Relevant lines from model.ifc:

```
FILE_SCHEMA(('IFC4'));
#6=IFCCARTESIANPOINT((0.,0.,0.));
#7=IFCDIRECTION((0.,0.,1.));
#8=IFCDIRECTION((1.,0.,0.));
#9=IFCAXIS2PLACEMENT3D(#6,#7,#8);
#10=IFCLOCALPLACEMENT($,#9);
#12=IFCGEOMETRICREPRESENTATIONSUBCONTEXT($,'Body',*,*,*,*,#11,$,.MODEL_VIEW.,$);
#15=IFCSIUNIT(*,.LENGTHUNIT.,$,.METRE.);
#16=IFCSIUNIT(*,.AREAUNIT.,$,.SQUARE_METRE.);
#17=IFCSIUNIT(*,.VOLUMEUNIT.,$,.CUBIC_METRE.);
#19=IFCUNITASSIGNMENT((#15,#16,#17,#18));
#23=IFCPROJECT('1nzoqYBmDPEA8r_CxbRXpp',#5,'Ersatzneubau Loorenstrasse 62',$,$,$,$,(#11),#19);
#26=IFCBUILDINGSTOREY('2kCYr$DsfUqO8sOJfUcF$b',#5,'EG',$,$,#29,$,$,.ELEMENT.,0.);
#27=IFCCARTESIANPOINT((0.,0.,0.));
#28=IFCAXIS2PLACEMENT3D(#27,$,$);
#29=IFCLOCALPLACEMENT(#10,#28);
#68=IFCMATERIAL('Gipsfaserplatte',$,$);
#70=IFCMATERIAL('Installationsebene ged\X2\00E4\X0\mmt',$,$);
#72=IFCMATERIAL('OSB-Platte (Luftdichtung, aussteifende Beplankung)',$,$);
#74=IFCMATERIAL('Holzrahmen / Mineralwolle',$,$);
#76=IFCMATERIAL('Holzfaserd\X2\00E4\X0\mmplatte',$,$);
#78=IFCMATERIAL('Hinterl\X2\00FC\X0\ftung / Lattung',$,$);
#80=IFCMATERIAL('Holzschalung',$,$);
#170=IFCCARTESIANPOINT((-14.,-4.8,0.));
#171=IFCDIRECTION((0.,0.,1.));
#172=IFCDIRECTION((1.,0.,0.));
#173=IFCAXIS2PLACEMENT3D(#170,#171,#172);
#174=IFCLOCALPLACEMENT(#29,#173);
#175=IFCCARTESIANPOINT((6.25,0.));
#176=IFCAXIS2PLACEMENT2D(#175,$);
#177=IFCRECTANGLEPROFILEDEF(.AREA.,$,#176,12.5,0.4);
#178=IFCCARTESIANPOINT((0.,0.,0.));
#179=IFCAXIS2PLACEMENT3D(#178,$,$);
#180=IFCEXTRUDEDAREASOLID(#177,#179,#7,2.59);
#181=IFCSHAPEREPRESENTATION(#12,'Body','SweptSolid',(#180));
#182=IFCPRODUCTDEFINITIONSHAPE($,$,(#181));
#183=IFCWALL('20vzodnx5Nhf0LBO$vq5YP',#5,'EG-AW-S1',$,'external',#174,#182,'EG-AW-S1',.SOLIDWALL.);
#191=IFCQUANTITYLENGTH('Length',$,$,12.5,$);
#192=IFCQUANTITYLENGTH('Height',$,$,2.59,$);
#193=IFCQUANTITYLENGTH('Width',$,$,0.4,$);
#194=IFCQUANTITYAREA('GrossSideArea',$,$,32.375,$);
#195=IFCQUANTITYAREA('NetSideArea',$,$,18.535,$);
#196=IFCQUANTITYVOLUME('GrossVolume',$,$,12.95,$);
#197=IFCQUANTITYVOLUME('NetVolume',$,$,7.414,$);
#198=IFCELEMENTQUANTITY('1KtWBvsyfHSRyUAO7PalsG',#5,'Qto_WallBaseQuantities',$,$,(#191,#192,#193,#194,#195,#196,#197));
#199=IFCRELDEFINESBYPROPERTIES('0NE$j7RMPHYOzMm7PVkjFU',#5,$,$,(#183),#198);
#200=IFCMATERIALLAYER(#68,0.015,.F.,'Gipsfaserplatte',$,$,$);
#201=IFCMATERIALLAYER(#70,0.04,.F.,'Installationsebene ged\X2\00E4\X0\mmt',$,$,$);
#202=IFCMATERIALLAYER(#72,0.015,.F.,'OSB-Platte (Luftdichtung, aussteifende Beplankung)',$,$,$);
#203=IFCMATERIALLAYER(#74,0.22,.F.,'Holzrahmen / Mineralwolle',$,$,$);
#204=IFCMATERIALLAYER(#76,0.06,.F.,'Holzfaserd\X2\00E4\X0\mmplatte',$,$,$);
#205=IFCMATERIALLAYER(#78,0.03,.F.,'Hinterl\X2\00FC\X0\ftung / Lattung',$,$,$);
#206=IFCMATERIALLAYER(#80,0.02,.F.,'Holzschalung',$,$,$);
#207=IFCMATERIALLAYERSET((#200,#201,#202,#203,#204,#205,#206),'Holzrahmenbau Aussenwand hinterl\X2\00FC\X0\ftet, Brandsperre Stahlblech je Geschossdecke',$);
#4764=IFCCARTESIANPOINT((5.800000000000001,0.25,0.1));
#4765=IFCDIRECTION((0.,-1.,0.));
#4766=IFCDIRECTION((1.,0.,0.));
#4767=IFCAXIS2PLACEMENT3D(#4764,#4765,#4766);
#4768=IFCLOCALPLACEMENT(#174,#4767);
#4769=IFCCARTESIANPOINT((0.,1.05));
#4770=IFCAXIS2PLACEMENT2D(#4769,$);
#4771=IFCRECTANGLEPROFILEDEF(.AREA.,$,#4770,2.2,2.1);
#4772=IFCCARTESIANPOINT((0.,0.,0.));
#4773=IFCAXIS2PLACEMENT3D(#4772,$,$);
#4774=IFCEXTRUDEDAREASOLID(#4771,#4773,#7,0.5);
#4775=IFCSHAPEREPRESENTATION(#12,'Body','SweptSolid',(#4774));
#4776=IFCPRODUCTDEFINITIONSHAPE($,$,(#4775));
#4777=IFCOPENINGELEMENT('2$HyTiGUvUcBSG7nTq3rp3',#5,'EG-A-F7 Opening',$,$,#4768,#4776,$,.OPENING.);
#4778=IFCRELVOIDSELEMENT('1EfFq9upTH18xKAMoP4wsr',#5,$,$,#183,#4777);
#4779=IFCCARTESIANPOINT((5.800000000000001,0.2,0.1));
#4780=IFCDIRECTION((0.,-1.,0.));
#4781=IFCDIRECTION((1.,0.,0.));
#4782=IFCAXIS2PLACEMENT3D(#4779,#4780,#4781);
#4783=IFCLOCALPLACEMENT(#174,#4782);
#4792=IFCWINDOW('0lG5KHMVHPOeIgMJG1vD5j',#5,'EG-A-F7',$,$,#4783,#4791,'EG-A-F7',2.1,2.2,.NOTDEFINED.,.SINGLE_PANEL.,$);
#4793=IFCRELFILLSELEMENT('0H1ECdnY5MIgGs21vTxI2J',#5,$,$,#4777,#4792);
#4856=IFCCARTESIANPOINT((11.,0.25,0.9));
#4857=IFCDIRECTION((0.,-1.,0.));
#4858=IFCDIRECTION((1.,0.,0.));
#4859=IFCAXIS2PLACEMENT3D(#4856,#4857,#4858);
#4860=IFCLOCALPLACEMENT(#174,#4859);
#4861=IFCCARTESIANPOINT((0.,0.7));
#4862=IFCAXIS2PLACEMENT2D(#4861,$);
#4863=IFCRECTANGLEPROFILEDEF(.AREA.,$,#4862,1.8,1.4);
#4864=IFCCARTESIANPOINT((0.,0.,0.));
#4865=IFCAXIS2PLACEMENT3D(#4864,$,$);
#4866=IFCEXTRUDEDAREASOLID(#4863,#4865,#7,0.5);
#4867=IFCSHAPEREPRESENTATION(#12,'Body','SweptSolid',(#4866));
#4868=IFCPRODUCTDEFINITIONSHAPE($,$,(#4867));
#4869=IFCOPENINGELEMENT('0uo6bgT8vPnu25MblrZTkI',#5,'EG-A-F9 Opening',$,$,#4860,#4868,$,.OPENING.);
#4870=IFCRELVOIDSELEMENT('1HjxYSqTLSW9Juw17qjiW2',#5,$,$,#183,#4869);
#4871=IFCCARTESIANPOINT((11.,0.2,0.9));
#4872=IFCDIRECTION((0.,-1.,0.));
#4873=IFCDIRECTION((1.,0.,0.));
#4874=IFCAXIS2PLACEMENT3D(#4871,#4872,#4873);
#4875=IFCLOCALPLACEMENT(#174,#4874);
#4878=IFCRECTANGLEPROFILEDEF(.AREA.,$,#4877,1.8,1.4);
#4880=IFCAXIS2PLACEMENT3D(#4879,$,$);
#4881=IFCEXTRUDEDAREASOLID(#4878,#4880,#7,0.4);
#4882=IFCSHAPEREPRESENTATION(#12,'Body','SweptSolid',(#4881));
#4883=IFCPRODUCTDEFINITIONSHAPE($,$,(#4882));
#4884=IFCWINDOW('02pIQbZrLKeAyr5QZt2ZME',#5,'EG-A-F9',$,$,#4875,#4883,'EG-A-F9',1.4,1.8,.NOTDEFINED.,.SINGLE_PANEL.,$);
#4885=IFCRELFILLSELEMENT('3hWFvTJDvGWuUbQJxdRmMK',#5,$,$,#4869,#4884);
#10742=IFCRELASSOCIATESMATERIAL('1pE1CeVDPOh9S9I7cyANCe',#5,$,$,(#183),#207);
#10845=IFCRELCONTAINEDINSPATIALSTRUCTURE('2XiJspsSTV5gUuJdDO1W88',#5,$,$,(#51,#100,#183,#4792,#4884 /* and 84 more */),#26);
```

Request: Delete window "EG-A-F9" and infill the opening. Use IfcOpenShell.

```python
import ifcopenshell
import ifcopenshell.api.feature
import ifcopenshell.api.pset
import ifcopenshell.api.root
import ifcopenshell.geom
import ifcopenshell.util.element
import ifcopenshell.util.shape
import ifcopenshell.util.unit

model = ifcopenshell.open("model.ifc")
area_scale = ifcopenshell.util.unit.calculate_unit_scale(model, "AREAUNIT")
volume_scale = ifcopenshell.util.unit.calculate_unit_scale(model, "VOLUMEUNIT")
settings = ifcopenshell.geom.settings()


def volume(element):
    """Net volume in cubic metres, openings subtracted."""
    shape = ifcopenshell.geom.create_shape(settings, element)
    return ifcopenshell.util.shape.get_volume(shape.geometry)


window = model.by_guid("02pIQbZrLKeAyr5QZt2ZME")
opening = window.FillsVoids[0].RelatingOpeningElement
wall = opening.VoidsElements[0].RelatingBuildingElement
before = volume(wall)

ifcopenshell.api.root.remove_product(model, product=window)
ifcopenshell.api.feature.remove_feature(model, feature=opening)

after = volume(wall)
thickness = 0.4  # wall thickness in metres

# Update the wall's stored quantities.
qto = model.by_id(ifcopenshell.util.element.get_pset(wall, "Qto_WallBaseQuantities", should_inherit=False)["id"])
ifcopenshell.api.pset.edit_qto(model, qto=qto, properties={
    "NetSideArea": after / thickness / area_scale,
    "NetVolume": after / volume_scale,
})

print(f"wall volume {before:.3f} -> {after:.3f} m3")

model.write("model_updated.ifc")
```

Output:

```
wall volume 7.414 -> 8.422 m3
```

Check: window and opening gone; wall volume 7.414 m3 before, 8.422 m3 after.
